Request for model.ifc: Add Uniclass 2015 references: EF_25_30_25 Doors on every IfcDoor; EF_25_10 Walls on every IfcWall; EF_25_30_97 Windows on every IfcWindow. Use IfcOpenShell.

First a look at what the model holds.

```python
import ifcopenshell

model = ifcopenshell.open("model.ifc")
print(model.schema)
print("classifications:", [c.Name for c in model.by_type("IfcClassification")])
for ifc_class in ("IfcDoor", "IfcRoof", "IfcStair", "IfcWall", "IfcWindow"):
    print(ifc_class, len(model.by_type(ifc_class)))
```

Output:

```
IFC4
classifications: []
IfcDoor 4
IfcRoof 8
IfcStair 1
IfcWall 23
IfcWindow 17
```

```python
import ifcopenshell
import ifcopenshell.api.classification

model = ifcopenshell.open("model.ifc")

system = ifcopenshell.api.classification.add_classification(model, classification="Uniclass 2015")

codes = {
    "IfcDoor": ("EF_25_30_25", "Doors"),
    "IfcWall": ("EF_25_10", "Walls"),
    "IfcWindow": ("EF_25_30_97", "Windows"),
}
for ifc_class, (code, name) in codes.items():
    products = model.by_type(ifc_class)
    ifcopenshell.api.classification.add_reference(
        model, products=products, classification=system, identification=code, name=name
    )
    print(code, len(products))

model.write("model_edited.ifc")
```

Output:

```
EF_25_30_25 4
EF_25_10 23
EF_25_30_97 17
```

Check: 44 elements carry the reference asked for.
